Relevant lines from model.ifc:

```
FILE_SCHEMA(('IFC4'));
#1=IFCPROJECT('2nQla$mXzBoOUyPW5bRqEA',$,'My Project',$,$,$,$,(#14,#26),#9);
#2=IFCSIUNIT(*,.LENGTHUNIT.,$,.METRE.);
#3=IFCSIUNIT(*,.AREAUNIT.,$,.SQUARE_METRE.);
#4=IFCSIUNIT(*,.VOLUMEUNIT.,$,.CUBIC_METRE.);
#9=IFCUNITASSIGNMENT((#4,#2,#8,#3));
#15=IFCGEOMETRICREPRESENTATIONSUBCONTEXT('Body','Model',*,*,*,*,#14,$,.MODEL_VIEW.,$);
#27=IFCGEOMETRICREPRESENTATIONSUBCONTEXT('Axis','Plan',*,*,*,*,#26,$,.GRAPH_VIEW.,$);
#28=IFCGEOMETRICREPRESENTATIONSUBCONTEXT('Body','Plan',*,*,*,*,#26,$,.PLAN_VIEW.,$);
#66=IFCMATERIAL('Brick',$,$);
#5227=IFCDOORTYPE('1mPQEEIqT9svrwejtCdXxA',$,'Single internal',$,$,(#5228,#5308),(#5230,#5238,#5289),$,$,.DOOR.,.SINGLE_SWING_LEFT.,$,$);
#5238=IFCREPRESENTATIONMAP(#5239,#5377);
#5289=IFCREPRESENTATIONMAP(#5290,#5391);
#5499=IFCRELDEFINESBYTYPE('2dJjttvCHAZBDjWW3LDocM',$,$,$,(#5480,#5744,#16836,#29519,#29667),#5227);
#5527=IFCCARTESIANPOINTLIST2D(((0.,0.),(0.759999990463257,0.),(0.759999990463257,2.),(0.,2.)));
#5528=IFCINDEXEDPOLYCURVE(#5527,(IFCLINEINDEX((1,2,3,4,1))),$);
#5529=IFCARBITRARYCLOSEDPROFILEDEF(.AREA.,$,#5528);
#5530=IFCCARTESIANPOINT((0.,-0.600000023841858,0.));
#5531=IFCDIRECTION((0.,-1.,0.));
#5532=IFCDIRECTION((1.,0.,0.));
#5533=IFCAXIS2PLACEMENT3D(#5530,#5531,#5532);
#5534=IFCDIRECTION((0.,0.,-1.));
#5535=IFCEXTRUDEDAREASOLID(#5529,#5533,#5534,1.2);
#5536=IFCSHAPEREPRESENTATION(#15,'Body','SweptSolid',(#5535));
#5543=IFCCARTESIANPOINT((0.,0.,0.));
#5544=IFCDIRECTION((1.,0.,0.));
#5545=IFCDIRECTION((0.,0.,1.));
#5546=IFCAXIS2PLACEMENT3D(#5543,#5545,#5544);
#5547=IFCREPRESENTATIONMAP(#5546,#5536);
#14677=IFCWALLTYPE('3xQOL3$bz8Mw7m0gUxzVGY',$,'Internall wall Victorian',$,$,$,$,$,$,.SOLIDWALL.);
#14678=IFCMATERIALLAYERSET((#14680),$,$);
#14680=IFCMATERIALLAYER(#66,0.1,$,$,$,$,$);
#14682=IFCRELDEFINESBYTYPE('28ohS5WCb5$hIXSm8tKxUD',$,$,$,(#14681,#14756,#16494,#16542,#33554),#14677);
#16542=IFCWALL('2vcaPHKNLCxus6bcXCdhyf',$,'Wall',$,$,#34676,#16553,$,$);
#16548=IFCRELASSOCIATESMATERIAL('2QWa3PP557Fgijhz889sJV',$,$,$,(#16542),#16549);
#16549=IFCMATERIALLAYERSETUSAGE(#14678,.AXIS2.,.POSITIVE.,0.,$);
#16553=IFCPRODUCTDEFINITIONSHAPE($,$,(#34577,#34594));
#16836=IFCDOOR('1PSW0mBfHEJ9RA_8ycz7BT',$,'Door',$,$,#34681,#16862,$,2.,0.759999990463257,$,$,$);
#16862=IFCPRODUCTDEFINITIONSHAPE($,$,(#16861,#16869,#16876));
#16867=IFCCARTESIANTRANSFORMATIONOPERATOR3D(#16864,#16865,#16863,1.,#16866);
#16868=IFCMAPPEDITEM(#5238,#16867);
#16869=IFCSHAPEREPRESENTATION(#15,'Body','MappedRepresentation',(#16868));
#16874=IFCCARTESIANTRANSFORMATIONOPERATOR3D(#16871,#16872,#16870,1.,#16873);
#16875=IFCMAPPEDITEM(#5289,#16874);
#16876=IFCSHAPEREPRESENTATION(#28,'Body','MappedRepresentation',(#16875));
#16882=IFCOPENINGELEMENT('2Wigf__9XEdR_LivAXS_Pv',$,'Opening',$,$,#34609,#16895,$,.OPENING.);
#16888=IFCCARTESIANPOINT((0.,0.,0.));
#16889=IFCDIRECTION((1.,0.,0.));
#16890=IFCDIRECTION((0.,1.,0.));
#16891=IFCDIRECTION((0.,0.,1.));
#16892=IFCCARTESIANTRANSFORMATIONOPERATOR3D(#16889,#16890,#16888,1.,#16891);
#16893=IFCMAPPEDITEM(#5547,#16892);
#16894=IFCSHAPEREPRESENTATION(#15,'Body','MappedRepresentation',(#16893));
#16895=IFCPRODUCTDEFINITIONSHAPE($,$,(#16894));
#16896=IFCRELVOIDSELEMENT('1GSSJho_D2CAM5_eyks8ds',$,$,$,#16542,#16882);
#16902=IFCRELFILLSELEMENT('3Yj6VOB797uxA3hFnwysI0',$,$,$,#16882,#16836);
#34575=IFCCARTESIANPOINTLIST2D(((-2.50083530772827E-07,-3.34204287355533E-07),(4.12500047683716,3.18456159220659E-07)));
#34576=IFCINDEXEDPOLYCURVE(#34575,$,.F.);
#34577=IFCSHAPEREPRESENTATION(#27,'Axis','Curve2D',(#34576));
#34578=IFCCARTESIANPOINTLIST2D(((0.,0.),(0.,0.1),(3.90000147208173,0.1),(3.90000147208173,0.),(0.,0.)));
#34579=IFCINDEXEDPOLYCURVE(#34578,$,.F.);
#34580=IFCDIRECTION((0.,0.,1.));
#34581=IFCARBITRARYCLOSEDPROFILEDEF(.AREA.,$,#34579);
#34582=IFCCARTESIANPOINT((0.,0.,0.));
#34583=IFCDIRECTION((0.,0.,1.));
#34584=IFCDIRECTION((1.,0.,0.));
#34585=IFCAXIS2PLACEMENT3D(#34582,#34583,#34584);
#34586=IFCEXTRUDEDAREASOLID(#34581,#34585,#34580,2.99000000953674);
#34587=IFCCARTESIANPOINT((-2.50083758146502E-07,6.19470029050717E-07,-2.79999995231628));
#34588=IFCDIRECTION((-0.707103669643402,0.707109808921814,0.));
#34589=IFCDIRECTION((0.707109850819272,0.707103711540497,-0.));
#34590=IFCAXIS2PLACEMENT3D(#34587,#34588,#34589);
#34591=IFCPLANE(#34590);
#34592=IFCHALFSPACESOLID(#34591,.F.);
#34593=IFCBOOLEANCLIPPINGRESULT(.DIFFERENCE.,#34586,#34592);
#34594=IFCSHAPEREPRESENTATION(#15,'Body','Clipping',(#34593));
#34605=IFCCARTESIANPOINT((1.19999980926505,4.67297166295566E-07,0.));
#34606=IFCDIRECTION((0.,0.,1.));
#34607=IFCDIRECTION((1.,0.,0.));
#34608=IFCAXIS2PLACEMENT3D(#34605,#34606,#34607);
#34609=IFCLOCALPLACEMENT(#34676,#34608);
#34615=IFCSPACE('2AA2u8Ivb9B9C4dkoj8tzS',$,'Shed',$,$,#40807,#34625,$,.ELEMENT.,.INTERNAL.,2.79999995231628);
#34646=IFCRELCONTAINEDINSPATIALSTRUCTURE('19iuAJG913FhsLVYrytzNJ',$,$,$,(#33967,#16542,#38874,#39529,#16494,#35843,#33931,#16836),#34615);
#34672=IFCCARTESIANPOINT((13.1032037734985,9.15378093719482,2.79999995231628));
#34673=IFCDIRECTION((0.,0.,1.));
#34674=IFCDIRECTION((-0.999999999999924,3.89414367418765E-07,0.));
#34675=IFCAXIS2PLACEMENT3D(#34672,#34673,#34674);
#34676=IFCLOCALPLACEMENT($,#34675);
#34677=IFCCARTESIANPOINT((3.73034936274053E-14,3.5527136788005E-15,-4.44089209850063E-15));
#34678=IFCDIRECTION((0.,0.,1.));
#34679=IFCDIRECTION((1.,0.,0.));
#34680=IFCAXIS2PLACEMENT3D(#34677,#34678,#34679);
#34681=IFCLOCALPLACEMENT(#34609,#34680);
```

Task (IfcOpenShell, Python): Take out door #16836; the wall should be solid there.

```python
import ifcopenshell
import ifcopenshell.api.feature
import ifcopenshell.api.root
import ifcopenshell.geom
import ifcopenshell.util.shape

model = ifcopenshell.open("model.ifc")
settings = ifcopenshell.geom.settings()


def volume(element):
    """Net volume in cubic metres, openings subtracted."""
    shape = ifcopenshell.geom.create_shape(settings, element)
    return ifcopenshell.util.shape.get_volume(shape.geometry)


door = model.by_guid("1PSW0mBfHEJ9RA_8ycz7BT")
opening = door.FillsVoids[0].RelatingOpeningElement
wall = opening.VoidsElements[0].RelatingBuildingElement
before = volume(wall)

ifcopenshell.api.root.remove_product(model, product=door)
ifcopenshell.api.feature.remove_feature(model, feature=opening)

after = volume(wall)

print(f"wall volume {before:.3f} -> {after:.3f} m3")

model.write("model_rev.ifc")
```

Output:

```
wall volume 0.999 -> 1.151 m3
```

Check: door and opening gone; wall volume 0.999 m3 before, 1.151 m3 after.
